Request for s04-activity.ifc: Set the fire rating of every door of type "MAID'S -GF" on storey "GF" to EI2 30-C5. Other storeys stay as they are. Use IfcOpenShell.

First a look at what the model holds.

```python
import ifcopenshell
import ifcopenshell.util.element

model = ifcopenshell.open("s04-activity.ifc")
print(model.schema)
storey = next(s for s in model.by_type("IfcBuildingStorey") if s.Name == "GF")
doors = [e for e in ifcopenshell.util.element.get_decomposition(storey) if e.is_a("IfcDoor")]
seen = {}
for e in doors:
    element_type = ifcopenshell.util.element.get_type(e)
    key = (element_type.Name if element_type != e and element_type else None, ifcopenshell.util.element.get_pset(e, "Pset_DoorCommon", "FireRating"))
    seen[key] = seen.get(key, 0) + 1
for (name, value), count in sorted(seen.items(), key=str):
    print(count, "x", name, "|", value)
```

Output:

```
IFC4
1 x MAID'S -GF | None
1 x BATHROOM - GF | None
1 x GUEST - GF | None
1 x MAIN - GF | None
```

```python
import ifcopenshell
import ifcopenshell.api.pset
import ifcopenshell.util.element

model = ifcopenshell.open("s04-activity.ifc")

storey = next(s for s in model.by_type("IfcBuildingStorey") if s.Name == "GF")
doors = [e for e in ifcopenshell.util.element.get_decomposition(storey) if e.is_a("IfcDoor")]

count = 0
for e in doors:
    element_type = ifcopenshell.util.element.get_type(e)
    if element_type in (None, e) or element_type.Name != "MAID'S -GF":
        continue
    # add_pset returns the element's existing set when there is one.
    pset = ifcopenshell.api.pset.add_pset(model, product=e, name="Pset_DoorCommon")
    ifcopenshell.api.pset.edit_pset(model, pset=pset, properties={"FireRating": "EI2 30-C5"})
    count += 1

print(count, "doors updated")

model.write("s04-activity_v2.ifc")
```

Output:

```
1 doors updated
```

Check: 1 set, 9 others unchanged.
